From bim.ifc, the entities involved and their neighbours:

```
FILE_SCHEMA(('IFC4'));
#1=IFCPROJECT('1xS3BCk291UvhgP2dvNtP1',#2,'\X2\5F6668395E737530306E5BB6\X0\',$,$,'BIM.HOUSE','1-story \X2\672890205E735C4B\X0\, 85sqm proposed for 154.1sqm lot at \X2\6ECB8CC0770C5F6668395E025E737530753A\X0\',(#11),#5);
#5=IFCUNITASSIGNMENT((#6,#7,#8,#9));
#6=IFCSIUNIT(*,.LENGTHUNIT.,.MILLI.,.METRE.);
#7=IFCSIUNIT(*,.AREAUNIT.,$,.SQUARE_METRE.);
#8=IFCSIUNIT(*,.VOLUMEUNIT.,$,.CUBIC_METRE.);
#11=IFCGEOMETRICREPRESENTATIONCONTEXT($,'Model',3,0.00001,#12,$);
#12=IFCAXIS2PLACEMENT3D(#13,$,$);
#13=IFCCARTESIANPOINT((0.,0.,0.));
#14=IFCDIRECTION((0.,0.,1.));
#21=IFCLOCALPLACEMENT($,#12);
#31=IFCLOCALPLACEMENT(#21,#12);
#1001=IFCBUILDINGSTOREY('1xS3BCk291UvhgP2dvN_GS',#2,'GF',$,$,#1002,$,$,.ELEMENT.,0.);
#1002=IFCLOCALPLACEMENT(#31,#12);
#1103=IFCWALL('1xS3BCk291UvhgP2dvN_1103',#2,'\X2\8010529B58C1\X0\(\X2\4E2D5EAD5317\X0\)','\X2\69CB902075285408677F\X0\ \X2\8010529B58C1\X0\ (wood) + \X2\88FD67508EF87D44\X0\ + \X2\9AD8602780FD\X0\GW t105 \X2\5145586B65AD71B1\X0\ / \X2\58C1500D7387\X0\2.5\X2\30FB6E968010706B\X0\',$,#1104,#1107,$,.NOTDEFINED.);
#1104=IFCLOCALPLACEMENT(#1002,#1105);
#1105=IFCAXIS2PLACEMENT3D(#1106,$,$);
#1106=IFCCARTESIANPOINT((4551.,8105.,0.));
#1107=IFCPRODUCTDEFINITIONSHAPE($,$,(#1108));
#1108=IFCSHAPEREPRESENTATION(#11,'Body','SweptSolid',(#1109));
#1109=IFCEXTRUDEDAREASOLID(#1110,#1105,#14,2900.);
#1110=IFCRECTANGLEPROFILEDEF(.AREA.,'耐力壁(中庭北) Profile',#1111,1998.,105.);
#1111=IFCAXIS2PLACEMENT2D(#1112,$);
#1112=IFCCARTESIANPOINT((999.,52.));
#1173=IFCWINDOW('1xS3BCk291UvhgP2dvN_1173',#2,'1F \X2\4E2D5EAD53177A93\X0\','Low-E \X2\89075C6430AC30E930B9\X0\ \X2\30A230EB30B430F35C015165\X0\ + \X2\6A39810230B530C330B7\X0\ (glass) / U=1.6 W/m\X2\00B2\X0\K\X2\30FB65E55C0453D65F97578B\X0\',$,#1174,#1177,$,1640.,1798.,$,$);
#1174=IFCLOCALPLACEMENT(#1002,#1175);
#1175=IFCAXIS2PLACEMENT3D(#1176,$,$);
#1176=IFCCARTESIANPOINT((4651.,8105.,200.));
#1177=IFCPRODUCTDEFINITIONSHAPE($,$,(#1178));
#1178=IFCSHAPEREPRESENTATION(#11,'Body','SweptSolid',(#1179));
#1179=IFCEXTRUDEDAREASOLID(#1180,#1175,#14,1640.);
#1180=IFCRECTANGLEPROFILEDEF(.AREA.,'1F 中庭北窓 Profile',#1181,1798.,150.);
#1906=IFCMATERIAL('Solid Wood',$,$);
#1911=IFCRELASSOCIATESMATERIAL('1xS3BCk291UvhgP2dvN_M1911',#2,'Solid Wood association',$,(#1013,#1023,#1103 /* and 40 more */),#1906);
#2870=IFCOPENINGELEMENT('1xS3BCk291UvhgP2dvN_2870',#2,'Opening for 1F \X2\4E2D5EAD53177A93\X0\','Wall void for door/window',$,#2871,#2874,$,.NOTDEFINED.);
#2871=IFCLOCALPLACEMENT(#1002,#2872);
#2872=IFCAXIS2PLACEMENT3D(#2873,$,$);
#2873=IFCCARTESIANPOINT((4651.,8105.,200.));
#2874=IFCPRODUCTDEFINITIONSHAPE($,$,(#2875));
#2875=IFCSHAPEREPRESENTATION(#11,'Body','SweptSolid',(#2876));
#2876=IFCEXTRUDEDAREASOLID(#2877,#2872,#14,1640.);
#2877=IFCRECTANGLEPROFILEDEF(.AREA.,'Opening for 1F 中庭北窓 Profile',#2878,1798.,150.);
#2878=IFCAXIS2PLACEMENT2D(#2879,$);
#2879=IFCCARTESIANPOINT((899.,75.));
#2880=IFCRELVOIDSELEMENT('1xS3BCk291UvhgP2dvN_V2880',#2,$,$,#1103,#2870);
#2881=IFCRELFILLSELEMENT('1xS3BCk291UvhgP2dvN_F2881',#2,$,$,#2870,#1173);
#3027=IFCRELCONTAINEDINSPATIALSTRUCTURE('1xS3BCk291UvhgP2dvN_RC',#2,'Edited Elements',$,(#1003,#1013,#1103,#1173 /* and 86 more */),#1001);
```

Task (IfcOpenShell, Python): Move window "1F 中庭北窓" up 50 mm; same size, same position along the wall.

```python
import numpy as np
import ifcopenshell
import ifcopenshell.api.geometry
import ifcopenshell.util.placement
import ifcopenshell.util.unit

model = ifcopenshell.open("bim.ifc")
unit_scale = ifcopenshell.util.unit.calculate_unit_scale(model)

window = model.by_guid("1xS3BCk291UvhgP2dvN_1173")
opening = window.FillsVoids[0].RelatingOpeningElement
dz = 0.05 / unit_scale

shift = np.array([0.0, 0.0, dz])
# The window is not placed relative to its opening, so move both.
for product in (opening, window):
    matrix = ifcopenshell.util.placement.get_local_placement(product.ObjectPlacement)
    matrix[:3, 3] += shift
    ifcopenshell.api.geometry.edit_object_placement(model, product=product, matrix=matrix, is_si=False)

print(f"moved by {dz * unit_scale:+.3f} m")

model.write("bim_edited.ifc")
```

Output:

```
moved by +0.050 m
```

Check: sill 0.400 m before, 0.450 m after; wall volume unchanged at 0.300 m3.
